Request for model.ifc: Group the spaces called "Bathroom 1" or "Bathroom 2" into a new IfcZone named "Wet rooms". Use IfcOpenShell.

First a look at what the model holds.

```python
import ifcopenshell

model = ifcopenshell.open("model.ifc")
print(model.schema)
seen = {}
for space in model.by_type("IfcSpace"):
    seen[space.LongName] = seen.get(space.LongName, 0) + 1
for name, count in sorted(seen.items(), key=str):
    print(count, "x", name)
print("zones:", [z.Name for z in model.by_type("IfcZone")][:20])
```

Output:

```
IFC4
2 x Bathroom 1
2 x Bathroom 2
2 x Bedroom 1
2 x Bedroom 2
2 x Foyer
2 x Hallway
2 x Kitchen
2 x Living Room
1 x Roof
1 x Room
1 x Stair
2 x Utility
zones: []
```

```python
import ifcopenshell
import ifcopenshell.api.group
import ifcopenshell.api.root

model = ifcopenshell.open("model.ifc")

names = {"Bathroom 1", "Bathroom 2"}
spaces = [s for s in model.by_type("IfcSpace") if s.LongName in names]

zone = ifcopenshell.api.root.create_entity(model, ifc_class="IfcZone", name="Wet rooms")
ifcopenshell.api.group.assign_group(model, products=spaces, group=zone)
print(len(spaces), "spaces in", zone.Name)

model.write("model_v2.ifc")
```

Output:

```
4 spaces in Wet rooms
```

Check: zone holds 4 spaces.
